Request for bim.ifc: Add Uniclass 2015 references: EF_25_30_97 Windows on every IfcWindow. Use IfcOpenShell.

First a look at what the model holds.

```python
import ifcopenshell

model = ifcopenshell.open("bim.ifc")
print(model.schema)
print("classifications:", [c.Name for c in model.by_type("IfcClassification")])
for ifc_class in ("IfcDoor", "IfcRoof", "IfcStair", "IfcWall", "IfcWindow"):
    print(ifc_class, len(model.by_type(ifc_class)))
```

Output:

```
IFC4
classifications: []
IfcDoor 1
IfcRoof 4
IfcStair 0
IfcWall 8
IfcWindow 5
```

```python
import ifcopenshell
import ifcopenshell.api.classification

model = ifcopenshell.open("bim.ifc")

system = ifcopenshell.api.classification.add_classification(model, classification="Uniclass 2015")

codes = {
    "IfcWindow": ("EF_25_30_97", "Windows"),
}
for ifc_class, (code, name) in codes.items():
    products = model.by_type(ifc_class)
    ifcopenshell.api.classification.add_reference(
        model, products=products, classification=system, identification=code, name=name
    )
    print(code, len(products))

model.write("bim_edited.ifc")
```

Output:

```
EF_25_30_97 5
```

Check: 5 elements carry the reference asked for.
